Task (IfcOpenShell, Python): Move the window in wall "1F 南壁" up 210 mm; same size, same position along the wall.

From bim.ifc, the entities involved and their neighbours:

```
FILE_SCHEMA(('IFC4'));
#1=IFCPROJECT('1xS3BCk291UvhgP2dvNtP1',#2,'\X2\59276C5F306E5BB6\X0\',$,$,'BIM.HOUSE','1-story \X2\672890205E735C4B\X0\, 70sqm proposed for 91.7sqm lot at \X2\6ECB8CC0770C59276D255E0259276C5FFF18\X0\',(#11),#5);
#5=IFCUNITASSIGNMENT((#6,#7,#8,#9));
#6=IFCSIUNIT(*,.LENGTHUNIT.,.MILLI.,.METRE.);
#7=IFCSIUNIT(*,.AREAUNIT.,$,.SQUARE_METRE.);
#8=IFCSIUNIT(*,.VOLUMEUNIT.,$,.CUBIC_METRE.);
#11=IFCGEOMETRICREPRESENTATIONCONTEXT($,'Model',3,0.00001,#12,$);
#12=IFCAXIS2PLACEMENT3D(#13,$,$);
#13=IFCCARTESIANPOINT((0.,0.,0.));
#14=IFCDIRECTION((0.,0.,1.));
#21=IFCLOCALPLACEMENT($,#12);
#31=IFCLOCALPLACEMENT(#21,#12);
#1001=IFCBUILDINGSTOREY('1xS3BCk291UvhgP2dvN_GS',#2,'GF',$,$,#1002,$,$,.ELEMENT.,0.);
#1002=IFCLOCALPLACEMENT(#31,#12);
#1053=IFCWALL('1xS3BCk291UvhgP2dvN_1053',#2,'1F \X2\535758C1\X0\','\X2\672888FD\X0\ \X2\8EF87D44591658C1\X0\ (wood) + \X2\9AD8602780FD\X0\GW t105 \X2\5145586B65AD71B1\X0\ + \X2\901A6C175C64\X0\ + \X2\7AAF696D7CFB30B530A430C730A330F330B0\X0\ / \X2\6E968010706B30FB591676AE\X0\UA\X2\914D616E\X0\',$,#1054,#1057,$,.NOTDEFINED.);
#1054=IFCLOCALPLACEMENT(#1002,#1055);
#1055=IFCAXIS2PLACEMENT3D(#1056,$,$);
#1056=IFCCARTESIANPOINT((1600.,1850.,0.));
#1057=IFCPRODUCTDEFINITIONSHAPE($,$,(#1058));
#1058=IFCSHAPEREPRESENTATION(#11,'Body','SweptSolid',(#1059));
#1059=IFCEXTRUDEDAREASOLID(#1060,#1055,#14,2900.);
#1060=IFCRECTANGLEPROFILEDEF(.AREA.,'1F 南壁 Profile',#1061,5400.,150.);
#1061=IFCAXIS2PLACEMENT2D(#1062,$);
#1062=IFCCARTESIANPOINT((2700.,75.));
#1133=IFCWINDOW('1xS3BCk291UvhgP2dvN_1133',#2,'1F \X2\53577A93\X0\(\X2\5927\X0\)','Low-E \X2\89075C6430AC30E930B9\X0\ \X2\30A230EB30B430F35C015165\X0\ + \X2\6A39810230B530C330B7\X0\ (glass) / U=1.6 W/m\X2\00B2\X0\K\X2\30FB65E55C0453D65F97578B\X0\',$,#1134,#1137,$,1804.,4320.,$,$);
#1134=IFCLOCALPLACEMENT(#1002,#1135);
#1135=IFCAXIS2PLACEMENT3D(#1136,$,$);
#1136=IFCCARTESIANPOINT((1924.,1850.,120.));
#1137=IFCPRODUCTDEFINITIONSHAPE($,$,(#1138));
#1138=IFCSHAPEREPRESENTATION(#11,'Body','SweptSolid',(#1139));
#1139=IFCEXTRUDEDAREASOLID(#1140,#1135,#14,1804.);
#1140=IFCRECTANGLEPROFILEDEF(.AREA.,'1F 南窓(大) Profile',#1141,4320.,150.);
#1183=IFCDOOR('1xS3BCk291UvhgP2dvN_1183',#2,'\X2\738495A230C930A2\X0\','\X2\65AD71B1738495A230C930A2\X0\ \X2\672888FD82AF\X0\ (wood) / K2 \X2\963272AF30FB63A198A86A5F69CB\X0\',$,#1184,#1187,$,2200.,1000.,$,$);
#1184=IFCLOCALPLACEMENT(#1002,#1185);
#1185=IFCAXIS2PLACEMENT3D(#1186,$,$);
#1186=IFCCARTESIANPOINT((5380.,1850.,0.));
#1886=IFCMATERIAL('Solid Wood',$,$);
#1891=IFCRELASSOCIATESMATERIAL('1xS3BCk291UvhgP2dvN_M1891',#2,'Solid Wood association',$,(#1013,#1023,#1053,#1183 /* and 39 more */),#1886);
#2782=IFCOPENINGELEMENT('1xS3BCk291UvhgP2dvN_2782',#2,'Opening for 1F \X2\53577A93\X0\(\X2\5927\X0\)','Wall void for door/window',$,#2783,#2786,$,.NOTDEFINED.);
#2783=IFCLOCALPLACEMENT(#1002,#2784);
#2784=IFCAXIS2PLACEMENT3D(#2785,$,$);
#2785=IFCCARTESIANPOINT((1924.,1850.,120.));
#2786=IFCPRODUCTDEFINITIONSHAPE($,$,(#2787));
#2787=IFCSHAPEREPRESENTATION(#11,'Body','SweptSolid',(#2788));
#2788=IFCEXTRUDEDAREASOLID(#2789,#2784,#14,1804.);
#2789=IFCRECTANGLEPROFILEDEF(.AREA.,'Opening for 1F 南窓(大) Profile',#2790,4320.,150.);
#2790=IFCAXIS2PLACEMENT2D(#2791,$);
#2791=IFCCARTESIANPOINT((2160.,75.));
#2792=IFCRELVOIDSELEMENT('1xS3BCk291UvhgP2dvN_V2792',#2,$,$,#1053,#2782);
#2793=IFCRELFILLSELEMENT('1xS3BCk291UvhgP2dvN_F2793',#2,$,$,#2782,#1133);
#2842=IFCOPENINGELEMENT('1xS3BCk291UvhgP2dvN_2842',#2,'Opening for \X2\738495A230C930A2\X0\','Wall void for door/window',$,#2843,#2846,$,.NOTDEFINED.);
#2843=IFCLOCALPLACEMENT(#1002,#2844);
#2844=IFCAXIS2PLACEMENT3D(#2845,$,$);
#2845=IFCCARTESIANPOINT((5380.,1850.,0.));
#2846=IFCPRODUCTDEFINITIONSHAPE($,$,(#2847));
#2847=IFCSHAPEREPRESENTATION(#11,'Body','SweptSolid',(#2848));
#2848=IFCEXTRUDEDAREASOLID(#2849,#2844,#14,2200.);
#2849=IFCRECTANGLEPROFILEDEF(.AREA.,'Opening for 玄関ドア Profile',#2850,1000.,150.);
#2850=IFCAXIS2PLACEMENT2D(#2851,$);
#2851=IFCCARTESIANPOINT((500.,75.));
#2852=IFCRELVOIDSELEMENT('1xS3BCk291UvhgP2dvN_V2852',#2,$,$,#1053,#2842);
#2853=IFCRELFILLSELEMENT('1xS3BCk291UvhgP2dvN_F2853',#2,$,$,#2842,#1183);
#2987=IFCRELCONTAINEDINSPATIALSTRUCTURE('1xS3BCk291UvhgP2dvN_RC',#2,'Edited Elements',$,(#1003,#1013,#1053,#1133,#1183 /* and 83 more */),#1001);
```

```python
import numpy as np
import ifcopenshell
import ifcopenshell.api.geometry
import ifcopenshell.util.placement
import ifcopenshell.util.unit

model = ifcopenshell.open("bim.ifc")
unit_scale = ifcopenshell.util.unit.calculate_unit_scale(model)

window = model.by_guid("1xS3BCk291UvhgP2dvN_1133")
opening = window.FillsVoids[0].RelatingOpeningElement
dz = 0.21 / unit_scale

shift = np.array([0.0, 0.0, dz])
# The window is not placed relative to its opening, so move both.
for product in (opening, window):
    matrix = ifcopenshell.util.placement.get_local_placement(product.ObjectPlacement)
    matrix[:3, 3] += shift
    ifcopenshell.api.geometry.edit_object_placement(model, product=product, matrix=matrix, is_si=False)

print(f"moved by {dz * unit_scale:+.3f} m")

model.write("bim_edited.ifc")
```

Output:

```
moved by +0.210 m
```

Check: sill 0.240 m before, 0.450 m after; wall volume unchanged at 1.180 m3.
